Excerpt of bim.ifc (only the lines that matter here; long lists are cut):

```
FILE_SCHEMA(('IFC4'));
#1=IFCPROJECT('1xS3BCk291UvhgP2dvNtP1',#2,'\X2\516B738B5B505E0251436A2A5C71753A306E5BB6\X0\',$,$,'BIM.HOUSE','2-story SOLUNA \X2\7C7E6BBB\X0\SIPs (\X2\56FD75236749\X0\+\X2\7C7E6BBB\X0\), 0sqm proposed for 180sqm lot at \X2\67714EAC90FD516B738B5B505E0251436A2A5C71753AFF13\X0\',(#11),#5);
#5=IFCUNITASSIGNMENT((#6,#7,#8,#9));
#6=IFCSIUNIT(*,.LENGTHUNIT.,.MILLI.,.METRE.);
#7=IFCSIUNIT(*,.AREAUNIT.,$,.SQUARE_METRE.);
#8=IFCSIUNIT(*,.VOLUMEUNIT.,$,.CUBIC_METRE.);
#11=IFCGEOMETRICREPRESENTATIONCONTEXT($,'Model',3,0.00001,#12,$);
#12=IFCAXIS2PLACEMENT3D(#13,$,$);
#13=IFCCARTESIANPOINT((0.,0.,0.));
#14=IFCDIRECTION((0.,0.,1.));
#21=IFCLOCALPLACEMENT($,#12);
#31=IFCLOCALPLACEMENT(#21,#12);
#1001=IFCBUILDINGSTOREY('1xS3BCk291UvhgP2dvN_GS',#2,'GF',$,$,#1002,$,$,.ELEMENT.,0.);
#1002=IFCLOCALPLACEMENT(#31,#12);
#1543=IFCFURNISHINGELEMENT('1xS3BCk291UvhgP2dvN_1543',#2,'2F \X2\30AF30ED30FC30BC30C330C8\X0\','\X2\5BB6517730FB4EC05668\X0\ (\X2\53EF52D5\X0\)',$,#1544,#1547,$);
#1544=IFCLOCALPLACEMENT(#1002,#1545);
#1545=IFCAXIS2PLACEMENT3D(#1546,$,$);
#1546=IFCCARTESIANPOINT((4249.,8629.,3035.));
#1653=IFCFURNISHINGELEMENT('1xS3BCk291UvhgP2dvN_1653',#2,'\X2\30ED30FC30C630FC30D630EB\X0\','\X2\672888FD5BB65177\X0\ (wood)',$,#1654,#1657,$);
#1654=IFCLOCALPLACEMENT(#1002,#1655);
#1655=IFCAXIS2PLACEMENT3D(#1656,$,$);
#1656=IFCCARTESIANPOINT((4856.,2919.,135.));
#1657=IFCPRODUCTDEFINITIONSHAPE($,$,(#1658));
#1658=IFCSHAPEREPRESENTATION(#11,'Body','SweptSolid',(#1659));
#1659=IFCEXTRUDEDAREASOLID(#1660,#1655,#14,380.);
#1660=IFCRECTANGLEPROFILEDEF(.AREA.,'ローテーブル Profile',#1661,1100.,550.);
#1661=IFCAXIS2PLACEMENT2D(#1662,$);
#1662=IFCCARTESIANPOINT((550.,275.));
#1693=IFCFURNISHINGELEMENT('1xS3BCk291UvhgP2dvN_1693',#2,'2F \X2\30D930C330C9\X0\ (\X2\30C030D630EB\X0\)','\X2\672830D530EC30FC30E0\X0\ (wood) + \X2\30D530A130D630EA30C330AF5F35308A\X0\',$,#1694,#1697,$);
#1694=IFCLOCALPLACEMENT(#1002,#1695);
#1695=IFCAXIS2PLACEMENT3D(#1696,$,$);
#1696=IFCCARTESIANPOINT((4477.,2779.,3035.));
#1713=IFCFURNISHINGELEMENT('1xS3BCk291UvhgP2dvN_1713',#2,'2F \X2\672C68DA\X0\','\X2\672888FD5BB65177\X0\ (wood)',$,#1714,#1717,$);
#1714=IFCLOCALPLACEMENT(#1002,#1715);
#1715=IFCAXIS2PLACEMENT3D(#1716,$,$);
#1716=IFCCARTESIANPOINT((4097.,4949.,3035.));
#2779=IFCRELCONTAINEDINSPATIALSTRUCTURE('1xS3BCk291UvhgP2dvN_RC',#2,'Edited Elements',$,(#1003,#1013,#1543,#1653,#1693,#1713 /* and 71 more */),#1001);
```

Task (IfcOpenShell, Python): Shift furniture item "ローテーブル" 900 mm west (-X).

```python
import ifcopenshell
import ifcopenshell.api.geometry
import ifcopenshell.util.placement
import ifcopenshell.util.unit

model = ifcopenshell.open("bim.ifc")
unit_scale = ifcopenshell.util.unit.calculate_unit_scale(model)

item = model.by_guid("1xS3BCk291UvhgP2dvN_1653")
matrix = ifcopenshell.util.placement.get_local_placement(item.ObjectPlacement)
matrix[0, 3] -= 0.9 / unit_scale
ifcopenshell.api.geometry.edit_object_placement(model, product=item, matrix=matrix, is_si=False)

print(ifcopenshell.util.placement.get_local_placement(item.ObjectPlacement).round(3) + 0.0)

model.write("bim_rev.ifc")
```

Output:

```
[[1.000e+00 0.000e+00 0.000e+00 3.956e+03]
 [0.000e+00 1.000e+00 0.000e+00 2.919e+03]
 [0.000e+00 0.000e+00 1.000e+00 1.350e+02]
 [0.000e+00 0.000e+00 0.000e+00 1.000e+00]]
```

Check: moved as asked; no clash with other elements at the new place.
